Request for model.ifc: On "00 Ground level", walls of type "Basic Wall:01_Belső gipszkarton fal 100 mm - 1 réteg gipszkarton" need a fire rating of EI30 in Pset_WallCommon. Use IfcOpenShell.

First a look at what the model holds.

```python
import ifcopenshell
import ifcopenshell.util.element

model = ifcopenshell.open("model.ifc")
print(model.schema)
storey = next(s for s in model.by_type("IfcBuildingStorey") if s.Name == "00 Ground level")
walls = [e for e in ifcopenshell.util.element.get_decomposition(storey) if e.is_a("IfcWall")]
seen = {}
for e in walls:
    element_type = ifcopenshell.util.element.get_type(e)
    key = (element_type.Name if element_type != e and element_type else None, ifcopenshell.util.element.get_pset(e, "Pset_WallCommon", "FireRating"))
    seen[key] = seen.get(key, 0) + 1
for (name, value), count in sorted(seen.items(), key=str):
    print(count, "x", name, "|", value)
```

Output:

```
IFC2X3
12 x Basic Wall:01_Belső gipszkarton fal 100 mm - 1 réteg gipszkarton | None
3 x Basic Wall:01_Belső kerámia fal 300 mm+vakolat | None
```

```python
import ifcopenshell
import ifcopenshell.api.pset
import ifcopenshell.util.element

model = ifcopenshell.open("model.ifc")

storey = next(s for s in model.by_type("IfcBuildingStorey") if s.Name == "00 Ground level")
walls = [e for e in ifcopenshell.util.element.get_decomposition(storey) if e.is_a("IfcWall")]

count = 0
for e in walls:
    element_type = ifcopenshell.util.element.get_type(e)
    if element_type in (None, e) or element_type.Name != "Basic Wall:01_Belső gipszkarton fal 100 mm - 1 réteg gipszkarton":
        continue
    # add_pset returns the element's existing set when there is one.
    pset = ifcopenshell.api.pset.add_pset(model, product=e, name="Pset_WallCommon")
    ifcopenshell.api.pset.edit_pset(model, pset=pset, properties={"FireRating": "EI30"})
    count += 1

print(count, "walls updated")

model.write("model_updated.ifc")
```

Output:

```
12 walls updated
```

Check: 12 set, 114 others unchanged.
